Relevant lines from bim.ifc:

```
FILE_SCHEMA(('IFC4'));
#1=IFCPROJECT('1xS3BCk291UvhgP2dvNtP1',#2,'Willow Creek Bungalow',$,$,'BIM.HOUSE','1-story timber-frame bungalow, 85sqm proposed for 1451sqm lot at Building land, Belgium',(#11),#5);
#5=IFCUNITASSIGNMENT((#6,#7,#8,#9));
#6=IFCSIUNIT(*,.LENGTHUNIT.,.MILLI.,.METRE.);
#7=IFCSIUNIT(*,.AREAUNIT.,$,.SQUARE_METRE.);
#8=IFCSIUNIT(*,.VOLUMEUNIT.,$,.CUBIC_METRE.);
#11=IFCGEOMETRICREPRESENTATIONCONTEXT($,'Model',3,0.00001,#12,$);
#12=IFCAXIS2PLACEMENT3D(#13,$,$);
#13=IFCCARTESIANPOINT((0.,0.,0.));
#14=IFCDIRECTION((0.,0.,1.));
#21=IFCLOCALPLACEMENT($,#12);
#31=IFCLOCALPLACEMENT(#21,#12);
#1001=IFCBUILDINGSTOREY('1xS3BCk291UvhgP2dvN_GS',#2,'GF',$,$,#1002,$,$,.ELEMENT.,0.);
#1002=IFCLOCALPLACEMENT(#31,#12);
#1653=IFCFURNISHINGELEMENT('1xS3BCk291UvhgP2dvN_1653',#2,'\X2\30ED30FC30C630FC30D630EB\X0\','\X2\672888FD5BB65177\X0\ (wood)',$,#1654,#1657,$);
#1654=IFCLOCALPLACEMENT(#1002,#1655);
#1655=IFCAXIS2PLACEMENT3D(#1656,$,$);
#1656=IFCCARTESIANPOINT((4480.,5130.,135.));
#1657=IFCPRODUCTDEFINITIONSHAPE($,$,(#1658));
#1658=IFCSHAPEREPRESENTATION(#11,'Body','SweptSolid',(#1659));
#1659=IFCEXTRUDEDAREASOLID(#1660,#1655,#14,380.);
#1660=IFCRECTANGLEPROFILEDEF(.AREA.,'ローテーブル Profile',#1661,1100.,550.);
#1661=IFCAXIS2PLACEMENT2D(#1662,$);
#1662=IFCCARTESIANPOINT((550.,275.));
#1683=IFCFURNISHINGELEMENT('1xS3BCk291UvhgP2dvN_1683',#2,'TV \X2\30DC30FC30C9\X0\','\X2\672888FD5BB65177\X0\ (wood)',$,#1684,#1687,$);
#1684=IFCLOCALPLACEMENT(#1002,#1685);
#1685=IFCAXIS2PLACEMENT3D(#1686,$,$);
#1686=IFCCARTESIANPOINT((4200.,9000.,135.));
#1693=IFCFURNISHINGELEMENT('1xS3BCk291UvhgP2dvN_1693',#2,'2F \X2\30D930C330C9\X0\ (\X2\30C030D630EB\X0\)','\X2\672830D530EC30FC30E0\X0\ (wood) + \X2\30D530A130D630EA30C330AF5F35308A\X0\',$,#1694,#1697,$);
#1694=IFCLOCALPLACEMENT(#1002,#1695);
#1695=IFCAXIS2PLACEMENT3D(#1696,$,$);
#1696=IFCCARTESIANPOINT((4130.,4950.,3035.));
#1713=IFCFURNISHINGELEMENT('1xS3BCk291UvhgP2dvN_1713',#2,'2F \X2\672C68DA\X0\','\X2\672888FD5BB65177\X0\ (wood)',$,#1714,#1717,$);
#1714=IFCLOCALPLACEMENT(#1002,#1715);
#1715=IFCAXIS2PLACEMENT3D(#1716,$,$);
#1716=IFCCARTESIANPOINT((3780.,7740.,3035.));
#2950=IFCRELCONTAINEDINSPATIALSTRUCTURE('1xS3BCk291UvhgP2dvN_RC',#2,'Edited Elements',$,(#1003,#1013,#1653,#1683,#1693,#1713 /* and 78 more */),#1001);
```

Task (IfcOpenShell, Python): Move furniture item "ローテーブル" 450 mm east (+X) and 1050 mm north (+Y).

```python
import ifcopenshell
import ifcopenshell.api.geometry
import ifcopenshell.util.placement
import ifcopenshell.util.unit

model = ifcopenshell.open("bim.ifc")
unit_scale = ifcopenshell.util.unit.calculate_unit_scale(model)

item = model.by_id(1653)
matrix = ifcopenshell.util.placement.get_local_placement(item.ObjectPlacement)
matrix[0, 3] += 0.45 / unit_scale
matrix[1, 3] += 1.05 / unit_scale
ifcopenshell.api.geometry.edit_object_placement(model, product=item, matrix=matrix, is_si=False)

print(ifcopenshell.util.placement.get_local_placement(item.ObjectPlacement).round(3) + 0.0)

model.write("bim_edited.ifc")
```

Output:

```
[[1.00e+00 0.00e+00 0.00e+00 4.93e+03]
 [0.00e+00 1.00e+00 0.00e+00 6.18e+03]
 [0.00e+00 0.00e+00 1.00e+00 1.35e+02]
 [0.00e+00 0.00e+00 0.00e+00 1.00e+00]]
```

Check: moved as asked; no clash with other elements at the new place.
